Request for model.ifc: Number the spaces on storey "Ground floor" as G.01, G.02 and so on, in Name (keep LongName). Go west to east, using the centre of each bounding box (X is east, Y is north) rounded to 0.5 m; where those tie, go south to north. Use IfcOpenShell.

First a look at what the model holds.

```python
import ifcopenshell
import ifcopenshell.util.element
import ifcopenshell.util.placement

model = ifcopenshell.open("model.ifc")
print(model.schema)
storey = next(s for s in model.by_type("IfcBuildingStorey") if s.Name == "Ground floor")
spaces = [e for e in ifcopenshell.util.element.get_decomposition(storey) if e.is_a("IfcSpace")]
for e in sorted(spaces, key=lambda e: e.id()):
    origin = ifcopenshell.util.placement.get_local_placement(e.ObjectPlacement)[:3, 3]
    print(e.id(), e.Name, e.LongName, origin.round(2) + 0.0, sep=" | ")
```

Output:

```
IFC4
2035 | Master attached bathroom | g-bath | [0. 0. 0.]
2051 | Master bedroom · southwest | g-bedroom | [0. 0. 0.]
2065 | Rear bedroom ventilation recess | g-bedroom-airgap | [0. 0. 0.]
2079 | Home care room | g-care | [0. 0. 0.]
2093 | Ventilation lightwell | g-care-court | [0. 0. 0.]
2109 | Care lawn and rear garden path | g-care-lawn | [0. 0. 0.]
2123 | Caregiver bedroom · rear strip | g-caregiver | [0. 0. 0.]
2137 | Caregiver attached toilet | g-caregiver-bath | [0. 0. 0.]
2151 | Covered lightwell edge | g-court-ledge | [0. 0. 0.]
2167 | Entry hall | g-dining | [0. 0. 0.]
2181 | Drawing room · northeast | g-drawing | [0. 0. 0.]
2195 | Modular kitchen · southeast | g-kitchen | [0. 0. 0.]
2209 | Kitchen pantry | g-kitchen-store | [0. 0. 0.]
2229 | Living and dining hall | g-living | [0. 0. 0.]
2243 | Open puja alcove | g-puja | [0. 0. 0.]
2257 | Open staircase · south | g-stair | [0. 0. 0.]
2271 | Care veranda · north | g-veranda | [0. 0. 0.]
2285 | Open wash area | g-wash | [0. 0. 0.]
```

```python
import ifcopenshell
import ifcopenshell.geom
import ifcopenshell.util.element
import ifcopenshell.util.shape

model = ifcopenshell.open("model.ifc")
settings = ifcopenshell.geom.settings()
settings.set("use-world-coords", True)


def centre(element):
    shape = ifcopenshell.geom.create_shape(settings, element)
    return ifcopenshell.util.shape.get_bbox_centroid(shape.geometry)


storey = next(s for s in model.by_type("IfcBuildingStorey") if s.Name == "Ground floor")
spaces = [e for e in ifcopenshell.util.element.get_decomposition(storey) if e.is_a("IfcSpace")]

# Insertion points can sit at a corner or the storey origin, so sort by the geometry (in metres).
centres = {e: centre(e) for e in spaces}
spaces.sort(key=lambda e: (round(centres[e][0] / 0.5), centres[e][1]))

for i, e in enumerate(spaces, start=1):
    number = f"G.{i:02d}"
    e.Name = number
    print(e.id(), number)

model.write("model_rev.ifc")
```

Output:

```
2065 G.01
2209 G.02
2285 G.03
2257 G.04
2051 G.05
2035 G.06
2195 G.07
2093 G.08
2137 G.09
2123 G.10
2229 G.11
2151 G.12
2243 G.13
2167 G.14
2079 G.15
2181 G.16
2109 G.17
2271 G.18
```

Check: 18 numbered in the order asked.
